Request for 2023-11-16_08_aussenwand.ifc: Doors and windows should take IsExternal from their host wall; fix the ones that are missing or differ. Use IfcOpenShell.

First a look at what the model holds.

```python
import ifcopenshell
import ifcopenshell.util.element

model = ifcopenshell.open("2023-11-16_08_aussenwand.ifc")
print(model.schema)
seen = {}
for e in model.by_type("IfcDoor") + model.by_type("IfcWindow"):
    if not e.FillsVoids:
        continue
    host = e.FillsVoids[0].RelatingOpeningElement.VoidsElements[0].RelatingBuildingElement
    own = ifcopenshell.util.element.get_pset(e, f"Pset_{e.is_a()[3:].removesuffix('StandardCase')}Common", "IsExternal")
    wall = ifcopenshell.util.element.get_pset(host, "Pset_WallCommon", "IsExternal")
    seen[e.is_a(), own, wall] = seen.get((e.is_a(), own, wall), 0) + 1
for (cls, own, wall), count in sorted(seen.items(), key=str):
    print(count, cls, "IsExternal:", own, "| host wall:", wall)
```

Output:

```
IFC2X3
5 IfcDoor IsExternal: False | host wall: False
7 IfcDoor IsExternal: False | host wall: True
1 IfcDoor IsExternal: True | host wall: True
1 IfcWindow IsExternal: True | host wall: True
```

```python
import ifcopenshell
import ifcopenshell.api.pset
import ifcopenshell.util.element

model = ifcopenshell.open("2023-11-16_08_aussenwand.ifc")

count = 0
for ifc_class, pset_name in (("IfcDoor", "Pset_DoorCommon"), ("IfcWindow", "Pset_WindowCommon")):
    for e in model.by_type(ifc_class):
        if not e.FillsVoids:
            continue
        host = e.FillsVoids[0].RelatingOpeningElement.VoidsElements[0].RelatingBuildingElement
        external = ifcopenshell.util.element.get_pset(host, "Pset_WallCommon", "IsExternal")
        if external is None or ifcopenshell.util.element.get_pset(e, pset_name, "IsExternal") == external:
            continue
        pset = ifcopenshell.api.pset.add_pset(model, product=e, name=pset_name)
        ifcopenshell.api.pset.edit_pset(model, pset=pset, properties={"IsExternal": external})
        count += 1

print(count, "updated")

model.write("2023-11-16_08_aussenwand-out.ifc")
```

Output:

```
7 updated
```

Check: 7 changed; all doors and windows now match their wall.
